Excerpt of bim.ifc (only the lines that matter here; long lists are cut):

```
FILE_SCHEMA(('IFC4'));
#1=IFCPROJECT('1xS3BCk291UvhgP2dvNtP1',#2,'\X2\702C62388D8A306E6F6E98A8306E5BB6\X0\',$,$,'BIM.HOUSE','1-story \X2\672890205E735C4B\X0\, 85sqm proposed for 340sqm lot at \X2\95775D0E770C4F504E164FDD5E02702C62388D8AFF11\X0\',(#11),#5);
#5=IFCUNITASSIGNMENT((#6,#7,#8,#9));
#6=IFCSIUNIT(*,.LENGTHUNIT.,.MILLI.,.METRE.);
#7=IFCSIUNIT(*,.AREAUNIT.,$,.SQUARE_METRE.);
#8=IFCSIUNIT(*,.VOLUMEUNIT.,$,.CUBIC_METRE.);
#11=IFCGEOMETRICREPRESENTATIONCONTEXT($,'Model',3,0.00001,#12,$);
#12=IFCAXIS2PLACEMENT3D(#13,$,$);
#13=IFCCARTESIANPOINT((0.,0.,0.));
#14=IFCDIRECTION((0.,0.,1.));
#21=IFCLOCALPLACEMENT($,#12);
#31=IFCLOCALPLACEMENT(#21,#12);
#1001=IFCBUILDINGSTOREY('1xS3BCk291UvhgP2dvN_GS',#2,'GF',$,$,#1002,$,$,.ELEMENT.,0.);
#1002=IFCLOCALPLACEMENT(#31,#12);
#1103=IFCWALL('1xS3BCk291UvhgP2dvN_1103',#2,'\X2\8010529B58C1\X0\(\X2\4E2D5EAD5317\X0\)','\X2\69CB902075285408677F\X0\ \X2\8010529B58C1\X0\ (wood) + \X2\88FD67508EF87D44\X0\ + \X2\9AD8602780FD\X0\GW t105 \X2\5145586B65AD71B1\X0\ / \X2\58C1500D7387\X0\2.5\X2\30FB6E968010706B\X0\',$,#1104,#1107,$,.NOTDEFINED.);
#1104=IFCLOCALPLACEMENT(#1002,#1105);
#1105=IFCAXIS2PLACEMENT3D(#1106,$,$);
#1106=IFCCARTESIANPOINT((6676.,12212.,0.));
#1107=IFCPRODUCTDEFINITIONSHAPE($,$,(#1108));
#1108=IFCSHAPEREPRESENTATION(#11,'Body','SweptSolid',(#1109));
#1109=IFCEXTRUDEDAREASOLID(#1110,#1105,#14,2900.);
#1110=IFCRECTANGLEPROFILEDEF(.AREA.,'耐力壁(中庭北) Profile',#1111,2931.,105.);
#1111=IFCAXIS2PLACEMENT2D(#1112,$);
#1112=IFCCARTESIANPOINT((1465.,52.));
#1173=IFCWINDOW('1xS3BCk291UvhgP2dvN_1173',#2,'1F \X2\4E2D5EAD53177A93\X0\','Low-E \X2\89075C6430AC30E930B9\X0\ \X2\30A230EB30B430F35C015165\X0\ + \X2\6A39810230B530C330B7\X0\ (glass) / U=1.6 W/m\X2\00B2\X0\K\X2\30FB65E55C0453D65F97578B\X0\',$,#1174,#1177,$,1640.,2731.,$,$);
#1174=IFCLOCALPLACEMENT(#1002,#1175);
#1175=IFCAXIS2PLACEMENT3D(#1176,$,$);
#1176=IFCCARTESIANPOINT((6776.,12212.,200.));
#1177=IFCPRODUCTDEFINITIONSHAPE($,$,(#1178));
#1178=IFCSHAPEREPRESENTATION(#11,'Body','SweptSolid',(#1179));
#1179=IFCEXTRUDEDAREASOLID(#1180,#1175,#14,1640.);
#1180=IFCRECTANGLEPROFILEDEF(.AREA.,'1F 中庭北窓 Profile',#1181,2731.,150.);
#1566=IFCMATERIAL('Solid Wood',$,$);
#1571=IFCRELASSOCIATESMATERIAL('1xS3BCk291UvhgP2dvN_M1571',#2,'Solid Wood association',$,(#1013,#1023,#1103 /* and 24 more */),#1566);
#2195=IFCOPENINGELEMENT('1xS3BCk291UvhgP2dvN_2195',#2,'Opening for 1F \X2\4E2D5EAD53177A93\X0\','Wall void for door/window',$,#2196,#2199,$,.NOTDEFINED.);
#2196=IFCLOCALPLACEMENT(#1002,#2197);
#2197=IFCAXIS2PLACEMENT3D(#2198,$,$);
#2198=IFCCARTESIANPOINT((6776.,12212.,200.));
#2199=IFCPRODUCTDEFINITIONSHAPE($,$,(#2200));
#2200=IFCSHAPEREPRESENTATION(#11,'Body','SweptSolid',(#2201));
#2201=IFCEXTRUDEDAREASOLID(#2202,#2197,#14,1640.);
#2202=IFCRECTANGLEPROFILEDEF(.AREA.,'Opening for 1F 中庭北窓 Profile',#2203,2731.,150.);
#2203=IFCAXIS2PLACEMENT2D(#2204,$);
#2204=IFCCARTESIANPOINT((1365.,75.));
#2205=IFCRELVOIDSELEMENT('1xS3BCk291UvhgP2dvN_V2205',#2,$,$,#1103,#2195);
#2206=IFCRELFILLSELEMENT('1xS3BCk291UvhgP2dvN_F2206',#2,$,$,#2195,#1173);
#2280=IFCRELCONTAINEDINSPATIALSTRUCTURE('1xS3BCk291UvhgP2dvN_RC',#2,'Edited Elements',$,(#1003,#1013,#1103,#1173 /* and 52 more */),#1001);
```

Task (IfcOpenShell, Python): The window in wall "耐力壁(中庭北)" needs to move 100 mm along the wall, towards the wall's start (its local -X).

```python
import ifcopenshell
import ifcopenshell.api.geometry
import ifcopenshell.util.placement

model = ifcopenshell.open("bim.ifc")

window = model.by_guid("1xS3BCk291UvhgP2dvN_1173")
opening = window.FillsVoids[0].RelatingOpeningElement
wall = opening.VoidsElements[0].RelatingBuildingElement

wall_matrix = ifcopenshell.util.placement.get_local_placement(wall.ObjectPlacement)
shift = wall_matrix[:3, 0] * -100.0
before = ifcopenshell.util.placement.get_local_placement(window.ObjectPlacement)[:3, 3].copy()

# The window is not placed relative to its opening, so move both.
for product in (opening, window):
    matrix = ifcopenshell.util.placement.get_local_placement(product.ObjectPlacement)
    matrix[:3, 3] += shift
    ifcopenshell.api.geometry.edit_object_placement(model, product=product, matrix=matrix, is_si=False)

after = ifcopenshell.util.placement.get_local_placement(window.ObjectPlacement)[:3, 3]
print("window moved by", (after - before).round(3) + 0.0)

model.write("bim_updated.ifc")
```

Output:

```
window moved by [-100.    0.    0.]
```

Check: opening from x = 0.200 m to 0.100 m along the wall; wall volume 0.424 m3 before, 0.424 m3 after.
